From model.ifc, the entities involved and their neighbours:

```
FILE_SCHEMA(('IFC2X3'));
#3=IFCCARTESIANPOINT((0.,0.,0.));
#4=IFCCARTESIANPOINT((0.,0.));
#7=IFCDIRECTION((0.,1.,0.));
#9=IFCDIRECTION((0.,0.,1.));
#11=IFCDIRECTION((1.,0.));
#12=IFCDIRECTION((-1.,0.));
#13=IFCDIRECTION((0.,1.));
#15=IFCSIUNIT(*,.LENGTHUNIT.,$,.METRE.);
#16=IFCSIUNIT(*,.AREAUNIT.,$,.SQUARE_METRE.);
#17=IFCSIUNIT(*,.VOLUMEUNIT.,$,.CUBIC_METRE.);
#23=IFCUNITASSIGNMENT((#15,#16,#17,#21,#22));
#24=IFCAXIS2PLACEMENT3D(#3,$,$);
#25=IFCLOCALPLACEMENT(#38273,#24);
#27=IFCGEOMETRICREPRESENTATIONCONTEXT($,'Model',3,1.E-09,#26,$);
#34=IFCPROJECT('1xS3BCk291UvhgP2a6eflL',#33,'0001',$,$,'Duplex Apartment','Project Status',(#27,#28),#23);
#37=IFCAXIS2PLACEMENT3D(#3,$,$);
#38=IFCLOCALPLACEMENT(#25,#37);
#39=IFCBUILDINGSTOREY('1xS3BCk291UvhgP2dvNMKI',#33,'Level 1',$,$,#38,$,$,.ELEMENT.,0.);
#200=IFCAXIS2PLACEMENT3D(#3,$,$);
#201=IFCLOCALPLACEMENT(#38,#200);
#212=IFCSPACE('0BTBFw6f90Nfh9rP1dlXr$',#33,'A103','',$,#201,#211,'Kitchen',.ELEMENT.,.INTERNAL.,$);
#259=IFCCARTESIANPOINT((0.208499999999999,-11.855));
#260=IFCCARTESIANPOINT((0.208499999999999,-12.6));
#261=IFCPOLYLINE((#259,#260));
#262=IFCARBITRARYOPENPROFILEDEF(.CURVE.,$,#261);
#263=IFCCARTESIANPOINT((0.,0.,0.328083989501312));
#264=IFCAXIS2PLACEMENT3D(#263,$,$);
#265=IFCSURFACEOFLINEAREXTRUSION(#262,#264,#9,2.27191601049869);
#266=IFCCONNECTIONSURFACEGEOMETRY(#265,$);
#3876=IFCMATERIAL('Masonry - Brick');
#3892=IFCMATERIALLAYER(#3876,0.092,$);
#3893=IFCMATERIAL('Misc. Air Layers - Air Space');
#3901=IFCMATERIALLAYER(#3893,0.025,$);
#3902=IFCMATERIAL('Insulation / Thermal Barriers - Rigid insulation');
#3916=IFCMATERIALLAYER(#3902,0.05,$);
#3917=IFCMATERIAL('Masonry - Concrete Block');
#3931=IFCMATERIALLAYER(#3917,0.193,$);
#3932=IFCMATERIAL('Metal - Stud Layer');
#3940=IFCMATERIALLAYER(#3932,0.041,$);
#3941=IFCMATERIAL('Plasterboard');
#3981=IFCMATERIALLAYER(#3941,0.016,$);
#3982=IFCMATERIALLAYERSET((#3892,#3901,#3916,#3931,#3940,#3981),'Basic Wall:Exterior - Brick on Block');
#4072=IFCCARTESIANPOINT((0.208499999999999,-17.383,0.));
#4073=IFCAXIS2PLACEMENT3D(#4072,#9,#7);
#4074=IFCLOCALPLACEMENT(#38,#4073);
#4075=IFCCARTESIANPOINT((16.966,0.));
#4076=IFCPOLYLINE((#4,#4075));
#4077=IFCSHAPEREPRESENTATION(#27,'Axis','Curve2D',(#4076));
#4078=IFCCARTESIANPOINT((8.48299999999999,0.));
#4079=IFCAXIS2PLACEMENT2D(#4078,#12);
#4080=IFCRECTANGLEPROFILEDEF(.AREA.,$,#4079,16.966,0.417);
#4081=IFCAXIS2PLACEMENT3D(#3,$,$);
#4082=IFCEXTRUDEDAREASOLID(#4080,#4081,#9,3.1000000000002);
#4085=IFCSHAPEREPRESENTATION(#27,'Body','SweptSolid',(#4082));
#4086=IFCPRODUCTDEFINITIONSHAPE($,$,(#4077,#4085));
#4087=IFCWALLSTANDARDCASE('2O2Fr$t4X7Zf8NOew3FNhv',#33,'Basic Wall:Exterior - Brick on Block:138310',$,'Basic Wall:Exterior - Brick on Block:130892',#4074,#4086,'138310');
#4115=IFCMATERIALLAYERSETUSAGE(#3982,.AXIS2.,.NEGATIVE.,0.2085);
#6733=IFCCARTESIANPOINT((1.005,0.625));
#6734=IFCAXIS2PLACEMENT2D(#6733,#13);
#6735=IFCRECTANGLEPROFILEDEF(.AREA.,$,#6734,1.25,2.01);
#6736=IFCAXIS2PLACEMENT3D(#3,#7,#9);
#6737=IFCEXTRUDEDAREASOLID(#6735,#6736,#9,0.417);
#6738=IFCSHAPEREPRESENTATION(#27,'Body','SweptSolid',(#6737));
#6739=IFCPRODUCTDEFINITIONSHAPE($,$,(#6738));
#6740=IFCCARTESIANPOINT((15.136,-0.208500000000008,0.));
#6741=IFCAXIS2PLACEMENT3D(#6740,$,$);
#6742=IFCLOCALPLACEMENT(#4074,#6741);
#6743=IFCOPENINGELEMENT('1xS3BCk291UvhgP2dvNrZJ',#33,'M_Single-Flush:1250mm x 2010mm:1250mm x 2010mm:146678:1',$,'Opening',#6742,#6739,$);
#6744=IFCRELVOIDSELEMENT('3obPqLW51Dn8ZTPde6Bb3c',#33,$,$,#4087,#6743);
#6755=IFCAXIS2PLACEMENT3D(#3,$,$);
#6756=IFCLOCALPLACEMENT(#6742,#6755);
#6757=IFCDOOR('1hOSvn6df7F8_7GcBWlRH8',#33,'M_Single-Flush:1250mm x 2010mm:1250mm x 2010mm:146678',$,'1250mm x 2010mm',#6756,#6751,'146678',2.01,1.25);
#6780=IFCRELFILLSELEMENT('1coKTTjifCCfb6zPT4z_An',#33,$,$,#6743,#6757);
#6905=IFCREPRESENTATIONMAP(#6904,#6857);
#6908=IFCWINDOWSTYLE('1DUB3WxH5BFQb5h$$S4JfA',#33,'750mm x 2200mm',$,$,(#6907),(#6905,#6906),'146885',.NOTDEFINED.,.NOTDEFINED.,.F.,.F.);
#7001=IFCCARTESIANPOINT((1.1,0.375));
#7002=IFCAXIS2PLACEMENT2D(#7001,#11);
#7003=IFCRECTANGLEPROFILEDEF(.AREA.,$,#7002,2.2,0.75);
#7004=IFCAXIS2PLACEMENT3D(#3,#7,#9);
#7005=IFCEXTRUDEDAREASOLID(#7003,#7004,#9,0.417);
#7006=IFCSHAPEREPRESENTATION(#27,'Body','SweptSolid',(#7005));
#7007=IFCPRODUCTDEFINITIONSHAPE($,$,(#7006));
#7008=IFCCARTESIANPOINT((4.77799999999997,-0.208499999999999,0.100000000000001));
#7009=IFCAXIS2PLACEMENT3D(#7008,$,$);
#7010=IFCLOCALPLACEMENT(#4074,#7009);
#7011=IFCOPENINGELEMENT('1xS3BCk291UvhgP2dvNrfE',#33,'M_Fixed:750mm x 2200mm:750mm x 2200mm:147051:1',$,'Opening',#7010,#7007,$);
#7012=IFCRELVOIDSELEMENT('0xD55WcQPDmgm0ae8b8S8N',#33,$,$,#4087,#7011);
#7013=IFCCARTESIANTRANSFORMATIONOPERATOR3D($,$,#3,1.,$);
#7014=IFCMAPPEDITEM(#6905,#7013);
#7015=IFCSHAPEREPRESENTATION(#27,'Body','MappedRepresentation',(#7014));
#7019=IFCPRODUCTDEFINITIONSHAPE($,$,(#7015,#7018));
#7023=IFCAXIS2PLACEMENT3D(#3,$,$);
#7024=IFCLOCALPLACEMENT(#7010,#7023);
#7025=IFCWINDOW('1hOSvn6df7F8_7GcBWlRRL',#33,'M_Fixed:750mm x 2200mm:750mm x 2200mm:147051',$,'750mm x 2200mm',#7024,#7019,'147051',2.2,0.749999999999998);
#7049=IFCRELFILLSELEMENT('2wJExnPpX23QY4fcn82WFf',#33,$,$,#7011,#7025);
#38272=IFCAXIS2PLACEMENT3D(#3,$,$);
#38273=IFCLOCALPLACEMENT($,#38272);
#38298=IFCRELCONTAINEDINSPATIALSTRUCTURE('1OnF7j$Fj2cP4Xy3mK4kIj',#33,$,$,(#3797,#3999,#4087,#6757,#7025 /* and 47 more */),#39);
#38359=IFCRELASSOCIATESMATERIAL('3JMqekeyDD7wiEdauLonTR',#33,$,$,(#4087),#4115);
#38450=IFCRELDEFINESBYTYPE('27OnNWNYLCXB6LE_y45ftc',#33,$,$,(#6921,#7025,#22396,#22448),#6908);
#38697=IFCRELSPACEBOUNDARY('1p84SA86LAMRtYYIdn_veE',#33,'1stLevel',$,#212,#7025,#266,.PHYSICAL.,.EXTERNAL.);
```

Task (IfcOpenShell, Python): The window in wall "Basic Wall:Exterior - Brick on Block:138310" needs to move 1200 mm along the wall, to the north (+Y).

```python
import numpy as np
import ifcopenshell
import ifcopenshell.api.geometry
import ifcopenshell.util.placement

model = ifcopenshell.open("model.ifc")

window = model.by_id(7025)
opening = window.FillsVoids[0].RelatingOpeningElement
wall = opening.VoidsElements[0].RelatingBuildingElement

wall_matrix = ifcopenshell.util.placement.get_local_placement(wall.ObjectPlacement)
shift = wall_matrix[:3, 0] * 1.2
before = ifcopenshell.util.placement.get_local_placement(window.ObjectPlacement)[:3, 3].copy()

# The window is placed relative to its opening, so it follows when the opening moves.
matrix = ifcopenshell.util.placement.get_local_placement(opening.ObjectPlacement)
matrix[:3, 3] += shift
ifcopenshell.api.geometry.edit_object_placement(
    model, product=opening, matrix=matrix, is_si=False, should_transform_children=True
)

# Space boundary surfaces are stored in each space's coordinates; move them too.
for rel in window.ProvidesBoundaries:
    if not rel.ConnectionGeometry:
        continue
    surface = rel.ConnectionGeometry.SurfaceOnRelatingElement
    space_matrix = ifcopenshell.util.placement.get_local_placement(rel.RelatingSpace.ObjectPlacement)
    point = np.array(surface.Position.Location.Coordinates) + space_matrix[:3, :3].T @ shift
    surface.Position = model.createIfcAxis2Placement3D(
        model.createIfcCartesianPoint(point.tolist()), surface.Position.Axis, surface.Position.RefDirection
    )

after = ifcopenshell.util.placement.get_local_placement(window.ObjectPlacement)[:3, 3]
print("window moved by", (after - before).round(3) + 0.0)

model.write("model_edited.ifc")
```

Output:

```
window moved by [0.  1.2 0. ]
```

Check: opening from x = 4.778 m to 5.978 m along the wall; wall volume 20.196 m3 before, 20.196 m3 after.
